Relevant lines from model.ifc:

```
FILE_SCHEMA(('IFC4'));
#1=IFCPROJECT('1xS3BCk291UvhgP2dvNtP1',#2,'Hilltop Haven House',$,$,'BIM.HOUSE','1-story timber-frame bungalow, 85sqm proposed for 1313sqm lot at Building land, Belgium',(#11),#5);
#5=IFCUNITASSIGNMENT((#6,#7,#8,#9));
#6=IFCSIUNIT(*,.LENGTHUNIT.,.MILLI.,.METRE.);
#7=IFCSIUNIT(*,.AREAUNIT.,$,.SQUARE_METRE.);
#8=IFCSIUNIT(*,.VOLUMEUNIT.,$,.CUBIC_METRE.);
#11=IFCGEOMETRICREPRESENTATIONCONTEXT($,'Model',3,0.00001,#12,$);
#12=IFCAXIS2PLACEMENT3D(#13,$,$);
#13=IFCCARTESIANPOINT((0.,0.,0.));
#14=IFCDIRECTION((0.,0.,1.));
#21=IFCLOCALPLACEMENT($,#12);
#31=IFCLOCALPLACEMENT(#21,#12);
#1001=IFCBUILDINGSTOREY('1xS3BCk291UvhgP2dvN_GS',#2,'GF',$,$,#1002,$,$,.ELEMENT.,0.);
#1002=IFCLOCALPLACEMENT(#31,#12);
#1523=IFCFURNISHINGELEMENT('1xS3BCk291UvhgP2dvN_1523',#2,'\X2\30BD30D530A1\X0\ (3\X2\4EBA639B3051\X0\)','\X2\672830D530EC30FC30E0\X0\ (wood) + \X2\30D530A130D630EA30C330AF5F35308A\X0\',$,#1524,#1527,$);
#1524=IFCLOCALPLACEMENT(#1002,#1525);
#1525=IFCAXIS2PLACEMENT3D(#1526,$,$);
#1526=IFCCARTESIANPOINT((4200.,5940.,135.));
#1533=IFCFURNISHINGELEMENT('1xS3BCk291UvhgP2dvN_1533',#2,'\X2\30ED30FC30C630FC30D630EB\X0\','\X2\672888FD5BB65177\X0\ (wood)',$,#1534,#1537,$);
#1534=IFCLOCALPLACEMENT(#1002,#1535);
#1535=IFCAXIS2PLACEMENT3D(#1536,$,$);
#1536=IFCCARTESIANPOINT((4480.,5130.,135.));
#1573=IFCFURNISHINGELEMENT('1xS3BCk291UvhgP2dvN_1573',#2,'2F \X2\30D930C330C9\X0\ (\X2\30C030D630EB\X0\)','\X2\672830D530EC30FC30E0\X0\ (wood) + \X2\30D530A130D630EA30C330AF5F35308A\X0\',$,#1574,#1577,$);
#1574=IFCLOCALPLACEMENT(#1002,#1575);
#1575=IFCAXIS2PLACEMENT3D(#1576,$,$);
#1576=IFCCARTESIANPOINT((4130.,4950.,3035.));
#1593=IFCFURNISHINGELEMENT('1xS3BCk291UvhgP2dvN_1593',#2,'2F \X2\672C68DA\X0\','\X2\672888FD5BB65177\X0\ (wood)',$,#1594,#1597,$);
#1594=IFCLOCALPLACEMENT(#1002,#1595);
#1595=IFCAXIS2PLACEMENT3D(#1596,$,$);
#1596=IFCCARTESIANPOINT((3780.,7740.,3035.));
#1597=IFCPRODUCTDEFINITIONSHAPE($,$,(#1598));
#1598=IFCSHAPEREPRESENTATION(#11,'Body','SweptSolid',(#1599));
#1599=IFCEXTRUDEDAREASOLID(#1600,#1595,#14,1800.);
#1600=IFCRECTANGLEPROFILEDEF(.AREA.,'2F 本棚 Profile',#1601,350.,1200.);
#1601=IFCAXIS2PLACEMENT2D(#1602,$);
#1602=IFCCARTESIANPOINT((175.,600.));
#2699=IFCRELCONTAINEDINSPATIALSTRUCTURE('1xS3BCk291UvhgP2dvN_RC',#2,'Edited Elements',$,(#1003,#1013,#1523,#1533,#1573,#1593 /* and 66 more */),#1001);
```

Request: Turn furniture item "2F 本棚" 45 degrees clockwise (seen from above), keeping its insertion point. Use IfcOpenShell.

```python
import ifcopenshell
import ifcopenshell.api.geometry
import ifcopenshell.util.placement

model = ifcopenshell.open("model.ifc")

item = model.by_id(1593)
matrix = ifcopenshell.util.placement.get_local_placement(item.ObjectPlacement)
matrix = matrix @ ifcopenshell.util.placement.rotation(-45, "Z")
ifcopenshell.api.geometry.edit_object_placement(model, product=item, matrix=matrix, is_si=False)

print(ifcopenshell.util.placement.get_local_placement(item.ObjectPlacement).round(3) + 0.0)

model.write("model_updated.ifc")
```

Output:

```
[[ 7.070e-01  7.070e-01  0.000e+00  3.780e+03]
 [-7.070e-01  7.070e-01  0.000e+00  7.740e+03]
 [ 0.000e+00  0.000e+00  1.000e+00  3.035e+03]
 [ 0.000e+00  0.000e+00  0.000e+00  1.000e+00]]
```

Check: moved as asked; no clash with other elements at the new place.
